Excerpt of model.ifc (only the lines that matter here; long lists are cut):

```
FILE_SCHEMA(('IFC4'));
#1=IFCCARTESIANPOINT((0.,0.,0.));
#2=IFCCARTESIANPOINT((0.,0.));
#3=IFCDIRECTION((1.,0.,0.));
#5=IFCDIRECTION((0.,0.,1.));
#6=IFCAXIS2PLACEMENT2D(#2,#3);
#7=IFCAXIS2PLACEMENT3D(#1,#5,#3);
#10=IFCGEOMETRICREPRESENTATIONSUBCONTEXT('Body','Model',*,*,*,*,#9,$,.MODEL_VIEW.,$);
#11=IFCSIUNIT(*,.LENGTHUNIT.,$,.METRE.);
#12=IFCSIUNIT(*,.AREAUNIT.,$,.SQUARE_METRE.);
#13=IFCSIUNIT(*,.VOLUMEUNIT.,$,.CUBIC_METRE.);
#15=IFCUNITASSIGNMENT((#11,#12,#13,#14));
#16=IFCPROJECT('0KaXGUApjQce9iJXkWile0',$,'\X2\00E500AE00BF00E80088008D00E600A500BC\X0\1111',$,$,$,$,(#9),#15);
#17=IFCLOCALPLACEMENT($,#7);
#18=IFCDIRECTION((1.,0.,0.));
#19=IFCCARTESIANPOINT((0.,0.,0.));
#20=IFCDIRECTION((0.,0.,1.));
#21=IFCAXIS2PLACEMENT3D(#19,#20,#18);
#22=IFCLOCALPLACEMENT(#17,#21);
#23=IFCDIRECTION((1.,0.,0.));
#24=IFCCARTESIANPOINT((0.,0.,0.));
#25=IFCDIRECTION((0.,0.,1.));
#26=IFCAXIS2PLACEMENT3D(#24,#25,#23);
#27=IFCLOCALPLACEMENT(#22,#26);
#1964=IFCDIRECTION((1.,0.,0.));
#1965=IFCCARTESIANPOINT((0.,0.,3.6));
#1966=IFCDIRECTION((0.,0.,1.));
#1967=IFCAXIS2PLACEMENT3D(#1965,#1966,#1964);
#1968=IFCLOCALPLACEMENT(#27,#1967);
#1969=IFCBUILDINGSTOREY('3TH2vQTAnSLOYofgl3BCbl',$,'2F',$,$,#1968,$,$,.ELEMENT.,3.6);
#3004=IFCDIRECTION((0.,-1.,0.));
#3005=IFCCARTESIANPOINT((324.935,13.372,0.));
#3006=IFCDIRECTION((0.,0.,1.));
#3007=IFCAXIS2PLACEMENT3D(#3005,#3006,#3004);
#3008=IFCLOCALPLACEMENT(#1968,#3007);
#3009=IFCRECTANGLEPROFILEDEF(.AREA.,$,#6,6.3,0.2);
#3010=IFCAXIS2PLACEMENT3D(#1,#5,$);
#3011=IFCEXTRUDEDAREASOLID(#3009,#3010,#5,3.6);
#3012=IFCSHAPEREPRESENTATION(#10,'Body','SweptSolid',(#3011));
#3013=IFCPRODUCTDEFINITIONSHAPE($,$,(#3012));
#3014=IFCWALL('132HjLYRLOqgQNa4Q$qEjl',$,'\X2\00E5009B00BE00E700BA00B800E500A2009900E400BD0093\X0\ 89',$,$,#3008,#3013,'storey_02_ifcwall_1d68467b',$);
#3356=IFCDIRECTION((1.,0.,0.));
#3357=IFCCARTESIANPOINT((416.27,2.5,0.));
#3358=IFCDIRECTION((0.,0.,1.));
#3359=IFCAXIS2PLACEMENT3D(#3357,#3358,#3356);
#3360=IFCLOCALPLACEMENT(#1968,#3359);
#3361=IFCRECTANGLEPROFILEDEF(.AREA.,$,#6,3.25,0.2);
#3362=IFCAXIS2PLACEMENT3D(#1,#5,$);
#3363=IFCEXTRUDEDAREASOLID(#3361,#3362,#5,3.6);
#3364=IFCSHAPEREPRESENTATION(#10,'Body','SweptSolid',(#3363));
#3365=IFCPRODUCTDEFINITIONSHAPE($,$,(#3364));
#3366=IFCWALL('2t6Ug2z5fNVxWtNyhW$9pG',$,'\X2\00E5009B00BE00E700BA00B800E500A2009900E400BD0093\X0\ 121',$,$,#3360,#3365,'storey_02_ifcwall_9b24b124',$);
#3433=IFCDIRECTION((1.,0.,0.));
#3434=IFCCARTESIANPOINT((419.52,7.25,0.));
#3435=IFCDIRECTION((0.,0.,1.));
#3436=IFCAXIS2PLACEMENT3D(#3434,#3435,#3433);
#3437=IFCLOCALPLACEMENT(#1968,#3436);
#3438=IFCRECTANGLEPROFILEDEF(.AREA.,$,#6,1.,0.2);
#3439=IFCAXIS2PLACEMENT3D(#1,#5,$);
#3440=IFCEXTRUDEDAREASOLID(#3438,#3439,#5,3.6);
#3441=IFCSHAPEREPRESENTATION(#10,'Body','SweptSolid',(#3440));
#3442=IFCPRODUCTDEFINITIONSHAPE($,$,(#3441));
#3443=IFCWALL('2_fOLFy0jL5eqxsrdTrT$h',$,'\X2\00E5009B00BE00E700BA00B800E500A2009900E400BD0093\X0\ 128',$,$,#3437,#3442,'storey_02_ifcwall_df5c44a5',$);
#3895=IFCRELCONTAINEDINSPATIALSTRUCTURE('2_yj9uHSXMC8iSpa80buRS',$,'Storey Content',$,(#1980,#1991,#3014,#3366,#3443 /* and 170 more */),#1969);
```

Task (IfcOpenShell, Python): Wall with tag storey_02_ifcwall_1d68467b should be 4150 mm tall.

```python
import ifcopenshell
import ifcopenshell.geom
import ifcopenshell.util.representation
import ifcopenshell.util.shape
import ifcopenshell.util.unit

model = ifcopenshell.open("model.ifc")
unit_scale = ifcopenshell.util.unit.calculate_unit_scale(model)
settings = ifcopenshell.geom.settings()


def volume(element):
    """Net volume in cubic metres, openings subtracted."""
    shape = ifcopenshell.geom.create_shape(settings, element)
    return ifcopenshell.util.shape.get_volume(shape.geometry)


wall = model.by_guid("132HjLYRLOqgQNa4Q$qEjl")
before = volume(wall)

body = ifcopenshell.util.representation.get_representation(wall, "Model", "Body")
solid = body.Items[0]
old_height = solid.Depth
solid.Depth = 4.15 / unit_scale
after = volume(wall)

print(f"height {old_height:g} -> {solid.Depth:g}, volume {before:.3f} -> {after:.3f} m3")

model.write("model_v2.ifc")
```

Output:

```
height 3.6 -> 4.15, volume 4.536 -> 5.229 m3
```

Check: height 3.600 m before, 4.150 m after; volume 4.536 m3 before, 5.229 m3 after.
